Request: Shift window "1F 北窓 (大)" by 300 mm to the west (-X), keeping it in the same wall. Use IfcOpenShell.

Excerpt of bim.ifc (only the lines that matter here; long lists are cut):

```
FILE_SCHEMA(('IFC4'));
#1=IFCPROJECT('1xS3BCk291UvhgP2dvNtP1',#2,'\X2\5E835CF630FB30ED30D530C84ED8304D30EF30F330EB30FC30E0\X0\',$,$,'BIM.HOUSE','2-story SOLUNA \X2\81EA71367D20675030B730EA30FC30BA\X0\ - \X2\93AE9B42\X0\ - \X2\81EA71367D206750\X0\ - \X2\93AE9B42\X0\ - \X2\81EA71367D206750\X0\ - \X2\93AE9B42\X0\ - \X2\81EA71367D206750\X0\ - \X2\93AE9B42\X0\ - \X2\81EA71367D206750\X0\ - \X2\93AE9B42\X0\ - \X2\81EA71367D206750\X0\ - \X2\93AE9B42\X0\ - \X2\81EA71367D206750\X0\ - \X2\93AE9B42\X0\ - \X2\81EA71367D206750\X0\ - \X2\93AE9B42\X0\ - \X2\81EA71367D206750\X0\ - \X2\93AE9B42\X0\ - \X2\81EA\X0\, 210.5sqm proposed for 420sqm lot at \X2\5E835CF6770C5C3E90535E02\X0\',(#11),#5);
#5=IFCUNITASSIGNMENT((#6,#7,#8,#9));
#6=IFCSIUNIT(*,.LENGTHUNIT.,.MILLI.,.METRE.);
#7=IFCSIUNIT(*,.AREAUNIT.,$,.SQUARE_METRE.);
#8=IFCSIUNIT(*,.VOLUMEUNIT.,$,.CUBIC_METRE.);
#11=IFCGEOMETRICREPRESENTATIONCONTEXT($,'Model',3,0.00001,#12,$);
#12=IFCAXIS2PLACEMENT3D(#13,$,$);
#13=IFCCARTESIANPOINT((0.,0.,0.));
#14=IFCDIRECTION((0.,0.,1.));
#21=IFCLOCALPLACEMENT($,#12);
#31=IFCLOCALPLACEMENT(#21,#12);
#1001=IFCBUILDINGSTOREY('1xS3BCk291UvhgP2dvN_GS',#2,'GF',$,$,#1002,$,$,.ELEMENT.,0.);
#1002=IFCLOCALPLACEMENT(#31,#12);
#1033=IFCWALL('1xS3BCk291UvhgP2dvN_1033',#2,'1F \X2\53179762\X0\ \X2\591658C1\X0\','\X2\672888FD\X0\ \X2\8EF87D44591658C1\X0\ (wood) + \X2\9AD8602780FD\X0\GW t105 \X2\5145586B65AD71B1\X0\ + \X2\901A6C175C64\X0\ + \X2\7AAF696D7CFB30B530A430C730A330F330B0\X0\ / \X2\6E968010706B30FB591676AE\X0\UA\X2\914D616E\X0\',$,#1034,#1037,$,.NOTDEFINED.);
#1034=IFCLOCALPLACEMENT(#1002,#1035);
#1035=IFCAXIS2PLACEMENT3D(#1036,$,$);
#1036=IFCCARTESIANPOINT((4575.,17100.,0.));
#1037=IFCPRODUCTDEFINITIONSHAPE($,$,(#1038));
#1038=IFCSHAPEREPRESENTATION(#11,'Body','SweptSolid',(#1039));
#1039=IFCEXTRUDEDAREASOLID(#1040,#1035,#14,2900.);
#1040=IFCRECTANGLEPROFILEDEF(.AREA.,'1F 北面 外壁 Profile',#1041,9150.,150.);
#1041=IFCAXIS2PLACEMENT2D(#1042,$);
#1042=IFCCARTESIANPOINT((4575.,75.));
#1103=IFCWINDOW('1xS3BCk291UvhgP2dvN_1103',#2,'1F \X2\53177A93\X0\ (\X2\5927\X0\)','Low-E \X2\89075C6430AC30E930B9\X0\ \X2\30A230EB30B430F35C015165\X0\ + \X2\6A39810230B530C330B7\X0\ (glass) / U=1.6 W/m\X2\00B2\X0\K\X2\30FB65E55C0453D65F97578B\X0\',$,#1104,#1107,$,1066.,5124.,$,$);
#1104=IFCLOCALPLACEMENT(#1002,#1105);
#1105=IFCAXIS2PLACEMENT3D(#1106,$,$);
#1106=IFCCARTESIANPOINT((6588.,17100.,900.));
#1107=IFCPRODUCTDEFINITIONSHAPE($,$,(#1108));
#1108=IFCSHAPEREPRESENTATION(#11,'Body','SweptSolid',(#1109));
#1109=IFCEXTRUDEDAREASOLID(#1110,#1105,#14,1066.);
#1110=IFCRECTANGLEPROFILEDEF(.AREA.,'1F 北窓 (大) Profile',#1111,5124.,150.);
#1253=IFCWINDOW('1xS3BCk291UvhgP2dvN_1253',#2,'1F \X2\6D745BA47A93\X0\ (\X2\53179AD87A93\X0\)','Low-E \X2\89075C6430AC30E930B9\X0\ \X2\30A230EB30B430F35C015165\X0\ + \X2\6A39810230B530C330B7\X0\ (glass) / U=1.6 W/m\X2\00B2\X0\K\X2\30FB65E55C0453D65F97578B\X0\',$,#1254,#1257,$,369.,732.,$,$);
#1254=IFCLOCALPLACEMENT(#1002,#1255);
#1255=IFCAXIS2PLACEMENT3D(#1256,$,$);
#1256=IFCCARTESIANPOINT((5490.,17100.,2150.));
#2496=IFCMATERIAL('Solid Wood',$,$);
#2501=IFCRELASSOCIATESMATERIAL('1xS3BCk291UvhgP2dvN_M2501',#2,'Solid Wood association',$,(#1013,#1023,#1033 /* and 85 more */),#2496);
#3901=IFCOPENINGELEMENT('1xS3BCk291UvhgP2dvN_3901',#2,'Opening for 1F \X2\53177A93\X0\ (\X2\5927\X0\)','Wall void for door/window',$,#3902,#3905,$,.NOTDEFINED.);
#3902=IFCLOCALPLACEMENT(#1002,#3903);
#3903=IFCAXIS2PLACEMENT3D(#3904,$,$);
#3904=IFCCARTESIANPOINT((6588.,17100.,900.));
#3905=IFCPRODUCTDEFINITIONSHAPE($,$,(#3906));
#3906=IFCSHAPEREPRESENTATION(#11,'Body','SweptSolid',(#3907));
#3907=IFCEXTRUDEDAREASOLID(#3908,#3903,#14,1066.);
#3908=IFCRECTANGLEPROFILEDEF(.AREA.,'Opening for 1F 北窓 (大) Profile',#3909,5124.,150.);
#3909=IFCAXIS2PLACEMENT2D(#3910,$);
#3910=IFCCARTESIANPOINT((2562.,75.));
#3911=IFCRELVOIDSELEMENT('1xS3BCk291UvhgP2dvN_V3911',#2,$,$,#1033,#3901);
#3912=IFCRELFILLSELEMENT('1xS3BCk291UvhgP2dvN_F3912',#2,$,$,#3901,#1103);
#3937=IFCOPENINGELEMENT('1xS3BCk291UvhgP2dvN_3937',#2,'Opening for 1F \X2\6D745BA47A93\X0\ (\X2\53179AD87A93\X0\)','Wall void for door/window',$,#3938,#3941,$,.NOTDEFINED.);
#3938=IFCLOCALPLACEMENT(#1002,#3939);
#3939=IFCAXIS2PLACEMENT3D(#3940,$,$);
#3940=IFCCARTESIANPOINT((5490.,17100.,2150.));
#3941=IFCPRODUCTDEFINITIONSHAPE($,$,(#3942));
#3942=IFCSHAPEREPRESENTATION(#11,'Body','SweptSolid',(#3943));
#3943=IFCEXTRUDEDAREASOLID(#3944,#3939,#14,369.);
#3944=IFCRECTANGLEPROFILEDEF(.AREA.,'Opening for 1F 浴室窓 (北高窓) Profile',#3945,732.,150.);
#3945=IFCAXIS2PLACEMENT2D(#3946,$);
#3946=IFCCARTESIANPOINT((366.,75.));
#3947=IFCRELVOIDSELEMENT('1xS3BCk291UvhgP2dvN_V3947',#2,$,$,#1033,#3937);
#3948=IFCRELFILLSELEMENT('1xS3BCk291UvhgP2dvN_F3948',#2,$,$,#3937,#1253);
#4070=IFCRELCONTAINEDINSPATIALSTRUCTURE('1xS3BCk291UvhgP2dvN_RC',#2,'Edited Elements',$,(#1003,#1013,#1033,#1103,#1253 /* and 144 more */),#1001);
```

```python
import ifcopenshell
import ifcopenshell.api.geometry
import ifcopenshell.util.placement

model = ifcopenshell.open("bim.ifc")

window = model.by_id(1103)
opening = window.FillsVoids[0].RelatingOpeningElement
wall = opening.VoidsElements[0].RelatingBuildingElement

wall_matrix = ifcopenshell.util.placement.get_local_placement(wall.ObjectPlacement)
shift = wall_matrix[:3, 0] * -300.0
before = ifcopenshell.util.placement.get_local_placement(window.ObjectPlacement)[:3, 3].copy()

# The window is not placed relative to its opening, so move both.
for product in (opening, window):
    matrix = ifcopenshell.util.placement.get_local_placement(product.ObjectPlacement)
    matrix[:3, 3] += shift
    ifcopenshell.api.geometry.edit_object_placement(model, product=product, matrix=matrix, is_si=False)

after = ifcopenshell.util.placement.get_local_placement(window.ObjectPlacement)[:3, 3]
print("window moved by", (after - before).round(3) + 0.0)

model.write("bim-out.ifc")
```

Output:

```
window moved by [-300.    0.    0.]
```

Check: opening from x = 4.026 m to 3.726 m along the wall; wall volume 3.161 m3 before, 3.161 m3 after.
